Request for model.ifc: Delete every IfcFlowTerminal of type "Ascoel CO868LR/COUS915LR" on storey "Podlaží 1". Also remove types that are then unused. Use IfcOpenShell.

First a look at what the model holds.

```python
import ifcopenshell
import ifcopenshell.util.element

model = ifcopenshell.open("model.ifc")
print(model.schema)
storey = next(s for s in model.by_type("IfcBuildingStorey") if s.Name == "Podlaží 1")
terminals = [e for e in ifcopenshell.util.element.get_decomposition(storey) if e.is_a("IfcFlowTerminal")]
seen = {}
for e in terminals:
    element_type = ifcopenshell.util.element.get_type(e)
    name = element_type.Name if element_type not in (None, e) else None
    seen[name] = seen.get(name, 0) + 1
for name, count in sorted(seen.items(), key=str):
    print(count, "x", name)
```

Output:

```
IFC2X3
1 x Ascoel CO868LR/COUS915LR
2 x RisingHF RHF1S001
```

```python
import ifcopenshell
import ifcopenshell.api.root
import ifcopenshell.util.element

model = ifcopenshell.open("model.ifc")

storey = next(s for s in model.by_type("IfcBuildingStorey") if s.Name == "Podlaží 1")
terminals = [e for e in ifcopenshell.util.element.get_decomposition(storey) if e.is_a("IfcFlowTerminal")]
targets = [e for e in terminals if (t := ifcopenshell.util.element.get_type(e)) not in (None, e) and t.Name == "Ascoel CO868LR/COUS915LR"]
types = {ifcopenshell.util.element.get_type(e) for e in targets} - {None, *targets}

for e in targets:
    ifcopenshell.api.root.remove_product(model, product=e)
print(len(targets), "removed")

unused = [t for t in types if not ifcopenshell.util.element.get_types(t)]
for t in unused:
    ifcopenshell.api.root.remove_product(model, product=t)
print(len(unused), "unused types removed")

model.write("model-out.ifc")
```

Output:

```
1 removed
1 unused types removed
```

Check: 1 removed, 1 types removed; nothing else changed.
